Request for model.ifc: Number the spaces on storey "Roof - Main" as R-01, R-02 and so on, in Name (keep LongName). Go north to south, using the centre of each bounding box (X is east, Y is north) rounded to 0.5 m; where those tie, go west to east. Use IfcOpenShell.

First a look at what the model holds.

```python
import ifcopenshell
import ifcopenshell.util.element
import ifcopenshell.util.placement

model = ifcopenshell.open("model.ifc")
print(model.schema)
storey = next(s for s in model.by_type("IfcBuildingStorey") if s.Name == "Roof - Main")
spaces = [e for e in ifcopenshell.util.element.get_decomposition(storey) if e.is_a("IfcSpace")]
for e in sorted(spaces, key=lambda e: e.id()):
    origin = ifcopenshell.util.placement.get_local_placement(e.ObjectPlacement)[:3, 3]
    print(e.id(), e.Name, e.LongName, origin.round(2) + 0.0, sep=" | ")
```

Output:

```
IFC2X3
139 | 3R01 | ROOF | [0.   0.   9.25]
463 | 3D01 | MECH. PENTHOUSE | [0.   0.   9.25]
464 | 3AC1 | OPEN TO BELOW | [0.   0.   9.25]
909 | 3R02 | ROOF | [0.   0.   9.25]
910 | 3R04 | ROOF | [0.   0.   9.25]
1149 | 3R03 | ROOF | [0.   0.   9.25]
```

```python
import ifcopenshell
import ifcopenshell.geom
import ifcopenshell.util.element
import ifcopenshell.util.shape

model = ifcopenshell.open("model.ifc")
settings = ifcopenshell.geom.settings()
settings.set("use-world-coords", True)


def centre(element):
    shape = ifcopenshell.geom.create_shape(settings, element)
    return ifcopenshell.util.shape.get_bbox_centroid(shape.geometry)


storey = next(s for s in model.by_type("IfcBuildingStorey") if s.Name == "Roof - Main")
spaces = [e for e in ifcopenshell.util.element.get_decomposition(storey) if e.is_a("IfcSpace")]

# Insertion points can sit at a corner or the storey origin, so sort by the geometry (in metres).
centres = {e: centre(e) for e in spaces}
spaces.sort(key=lambda e: (-round(centres[e][1] / 0.5), centres[e][0]))

for i, e in enumerate(spaces, start=1):
    number = f"R-{i:02d}"
    e.Name = number
    print(e.id(), number)

model.write("model-out.ifc")
```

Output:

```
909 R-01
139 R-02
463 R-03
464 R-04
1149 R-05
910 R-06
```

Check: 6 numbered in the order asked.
